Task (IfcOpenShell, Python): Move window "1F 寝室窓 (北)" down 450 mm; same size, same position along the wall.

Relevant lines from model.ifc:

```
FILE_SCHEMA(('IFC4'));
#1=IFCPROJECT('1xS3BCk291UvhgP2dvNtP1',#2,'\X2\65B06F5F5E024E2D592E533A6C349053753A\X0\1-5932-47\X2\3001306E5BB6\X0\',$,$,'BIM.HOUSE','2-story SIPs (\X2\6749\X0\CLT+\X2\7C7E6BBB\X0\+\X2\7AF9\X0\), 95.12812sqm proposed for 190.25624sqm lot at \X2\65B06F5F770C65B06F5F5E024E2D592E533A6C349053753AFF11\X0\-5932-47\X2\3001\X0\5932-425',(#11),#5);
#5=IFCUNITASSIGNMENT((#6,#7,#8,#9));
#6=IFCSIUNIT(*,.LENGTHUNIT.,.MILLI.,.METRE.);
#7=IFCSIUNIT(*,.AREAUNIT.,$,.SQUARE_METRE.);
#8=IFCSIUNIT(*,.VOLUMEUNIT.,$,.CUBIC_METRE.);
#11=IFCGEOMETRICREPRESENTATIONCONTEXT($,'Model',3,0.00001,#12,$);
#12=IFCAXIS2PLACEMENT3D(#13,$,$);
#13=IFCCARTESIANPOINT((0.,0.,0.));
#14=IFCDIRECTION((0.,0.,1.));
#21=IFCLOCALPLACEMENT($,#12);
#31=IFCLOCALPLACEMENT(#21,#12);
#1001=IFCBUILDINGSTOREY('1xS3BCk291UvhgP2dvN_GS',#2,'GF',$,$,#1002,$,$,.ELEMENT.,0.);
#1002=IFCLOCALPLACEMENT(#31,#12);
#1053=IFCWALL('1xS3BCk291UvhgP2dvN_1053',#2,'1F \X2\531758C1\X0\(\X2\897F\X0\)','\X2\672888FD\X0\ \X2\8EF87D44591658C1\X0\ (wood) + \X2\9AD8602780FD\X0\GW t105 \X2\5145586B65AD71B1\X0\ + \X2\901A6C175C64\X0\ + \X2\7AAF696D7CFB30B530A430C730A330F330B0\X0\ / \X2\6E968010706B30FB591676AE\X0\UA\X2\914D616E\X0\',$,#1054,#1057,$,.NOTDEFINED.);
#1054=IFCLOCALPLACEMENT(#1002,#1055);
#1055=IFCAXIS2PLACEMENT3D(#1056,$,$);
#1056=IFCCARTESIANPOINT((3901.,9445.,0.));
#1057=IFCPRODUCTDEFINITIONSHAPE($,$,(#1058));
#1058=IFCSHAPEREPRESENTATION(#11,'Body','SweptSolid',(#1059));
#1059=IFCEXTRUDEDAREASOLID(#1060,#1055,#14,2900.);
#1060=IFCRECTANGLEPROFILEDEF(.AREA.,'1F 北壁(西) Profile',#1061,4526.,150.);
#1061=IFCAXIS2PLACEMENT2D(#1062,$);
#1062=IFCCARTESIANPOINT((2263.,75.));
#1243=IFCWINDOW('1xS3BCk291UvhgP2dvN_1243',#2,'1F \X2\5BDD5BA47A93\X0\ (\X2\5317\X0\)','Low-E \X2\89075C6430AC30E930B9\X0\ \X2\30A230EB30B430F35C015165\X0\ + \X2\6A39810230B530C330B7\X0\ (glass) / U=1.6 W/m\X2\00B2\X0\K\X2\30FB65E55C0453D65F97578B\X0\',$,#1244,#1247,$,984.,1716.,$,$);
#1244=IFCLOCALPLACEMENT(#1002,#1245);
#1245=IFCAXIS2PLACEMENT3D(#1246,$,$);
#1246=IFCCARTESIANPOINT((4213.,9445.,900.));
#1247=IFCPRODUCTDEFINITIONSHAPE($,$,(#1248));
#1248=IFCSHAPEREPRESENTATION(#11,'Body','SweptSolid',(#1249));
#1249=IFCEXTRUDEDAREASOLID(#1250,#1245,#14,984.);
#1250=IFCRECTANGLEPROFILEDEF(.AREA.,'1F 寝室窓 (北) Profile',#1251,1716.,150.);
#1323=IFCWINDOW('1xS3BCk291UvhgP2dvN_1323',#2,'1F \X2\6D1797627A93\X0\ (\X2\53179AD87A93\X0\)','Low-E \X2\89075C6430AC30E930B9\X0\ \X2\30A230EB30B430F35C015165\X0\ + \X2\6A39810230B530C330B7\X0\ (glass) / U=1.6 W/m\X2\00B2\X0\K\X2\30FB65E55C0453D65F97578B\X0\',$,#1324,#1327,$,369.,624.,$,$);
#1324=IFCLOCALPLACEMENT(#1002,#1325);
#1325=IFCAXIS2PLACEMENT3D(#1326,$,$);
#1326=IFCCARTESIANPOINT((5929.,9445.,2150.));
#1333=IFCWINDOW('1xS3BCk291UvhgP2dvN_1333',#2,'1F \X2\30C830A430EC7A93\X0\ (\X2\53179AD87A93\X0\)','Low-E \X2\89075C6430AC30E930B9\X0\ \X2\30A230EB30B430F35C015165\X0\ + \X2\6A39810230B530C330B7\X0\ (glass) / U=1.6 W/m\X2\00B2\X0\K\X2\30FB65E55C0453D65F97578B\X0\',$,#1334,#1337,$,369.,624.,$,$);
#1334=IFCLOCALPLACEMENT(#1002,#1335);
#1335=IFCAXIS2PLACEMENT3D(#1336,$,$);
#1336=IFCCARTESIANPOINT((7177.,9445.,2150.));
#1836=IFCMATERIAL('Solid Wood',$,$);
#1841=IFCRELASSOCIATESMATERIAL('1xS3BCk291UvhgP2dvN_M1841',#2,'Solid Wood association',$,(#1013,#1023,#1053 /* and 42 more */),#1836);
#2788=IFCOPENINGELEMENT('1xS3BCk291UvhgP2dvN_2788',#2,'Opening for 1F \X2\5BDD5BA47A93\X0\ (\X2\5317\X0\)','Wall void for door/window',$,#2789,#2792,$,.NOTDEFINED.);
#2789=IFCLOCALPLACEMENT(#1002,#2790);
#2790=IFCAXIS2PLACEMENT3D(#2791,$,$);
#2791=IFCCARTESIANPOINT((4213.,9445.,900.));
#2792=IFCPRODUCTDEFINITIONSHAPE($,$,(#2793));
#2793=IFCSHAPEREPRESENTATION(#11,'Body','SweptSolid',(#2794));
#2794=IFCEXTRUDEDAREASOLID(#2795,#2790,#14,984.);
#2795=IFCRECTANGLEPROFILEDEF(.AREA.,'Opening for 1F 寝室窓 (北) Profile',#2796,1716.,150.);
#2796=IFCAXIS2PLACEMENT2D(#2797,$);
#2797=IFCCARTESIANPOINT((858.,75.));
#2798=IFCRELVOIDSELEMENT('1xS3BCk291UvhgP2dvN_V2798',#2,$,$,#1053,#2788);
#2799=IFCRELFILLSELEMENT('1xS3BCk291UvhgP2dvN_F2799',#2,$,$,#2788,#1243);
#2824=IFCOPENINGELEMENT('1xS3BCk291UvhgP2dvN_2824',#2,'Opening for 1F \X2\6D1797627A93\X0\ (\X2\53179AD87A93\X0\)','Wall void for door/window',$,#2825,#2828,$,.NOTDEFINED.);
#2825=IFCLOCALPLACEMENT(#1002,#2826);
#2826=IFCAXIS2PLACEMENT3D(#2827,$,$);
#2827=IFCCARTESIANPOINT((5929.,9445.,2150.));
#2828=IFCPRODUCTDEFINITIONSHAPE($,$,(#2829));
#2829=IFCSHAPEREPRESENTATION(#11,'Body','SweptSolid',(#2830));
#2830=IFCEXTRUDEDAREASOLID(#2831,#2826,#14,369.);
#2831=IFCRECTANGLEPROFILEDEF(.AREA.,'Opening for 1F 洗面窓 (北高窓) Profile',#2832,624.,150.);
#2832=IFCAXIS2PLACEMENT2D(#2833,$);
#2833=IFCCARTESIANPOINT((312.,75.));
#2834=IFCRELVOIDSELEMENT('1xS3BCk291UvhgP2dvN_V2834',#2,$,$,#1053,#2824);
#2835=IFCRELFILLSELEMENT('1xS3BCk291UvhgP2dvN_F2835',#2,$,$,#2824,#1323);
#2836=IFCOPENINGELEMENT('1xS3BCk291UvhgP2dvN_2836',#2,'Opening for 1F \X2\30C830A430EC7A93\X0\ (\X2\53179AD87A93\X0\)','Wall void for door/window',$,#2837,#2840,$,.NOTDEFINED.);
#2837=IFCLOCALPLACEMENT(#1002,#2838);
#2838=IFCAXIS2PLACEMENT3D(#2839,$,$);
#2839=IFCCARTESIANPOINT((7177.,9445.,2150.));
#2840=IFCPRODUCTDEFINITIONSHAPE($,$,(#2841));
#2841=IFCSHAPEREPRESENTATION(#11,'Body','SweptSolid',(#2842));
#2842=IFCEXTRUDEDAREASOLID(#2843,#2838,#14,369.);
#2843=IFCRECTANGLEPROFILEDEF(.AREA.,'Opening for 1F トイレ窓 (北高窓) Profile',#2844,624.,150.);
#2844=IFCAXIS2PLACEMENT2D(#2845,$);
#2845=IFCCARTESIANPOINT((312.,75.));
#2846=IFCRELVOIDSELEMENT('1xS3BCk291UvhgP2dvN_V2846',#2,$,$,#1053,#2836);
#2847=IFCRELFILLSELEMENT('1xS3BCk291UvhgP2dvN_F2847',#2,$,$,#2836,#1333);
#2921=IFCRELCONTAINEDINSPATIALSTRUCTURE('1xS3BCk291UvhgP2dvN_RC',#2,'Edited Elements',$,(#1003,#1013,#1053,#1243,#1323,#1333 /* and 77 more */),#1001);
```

```python
import numpy as np
import ifcopenshell
import ifcopenshell.api.geometry
import ifcopenshell.util.placement
import ifcopenshell.util.unit

model = ifcopenshell.open("model.ifc")
unit_scale = ifcopenshell.util.unit.calculate_unit_scale(model)

window = model.by_id(1243)
opening = window.FillsVoids[0].RelatingOpeningElement
dz = -0.45 / unit_scale

shift = np.array([0.0, 0.0, dz])
# The window is not placed relative to its opening, so move both.
for product in (opening, window):
    matrix = ifcopenshell.util.placement.get_local_placement(product.ObjectPlacement)
    matrix[:3, 3] += shift
    ifcopenshell.api.geometry.edit_object_placement(model, product=product, matrix=matrix, is_si=False)

print(f"moved by {dz * unit_scale:+.3f} m")

model.write("model_edited.ifc")
```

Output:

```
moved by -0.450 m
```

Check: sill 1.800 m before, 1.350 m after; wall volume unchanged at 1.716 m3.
